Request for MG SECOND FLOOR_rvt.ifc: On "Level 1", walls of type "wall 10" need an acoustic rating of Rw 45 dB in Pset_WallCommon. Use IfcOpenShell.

First a look at what the model holds.

```python
import ifcopenshell
import ifcopenshell.util.element

model = ifcopenshell.open("MG SECOND FLOOR_rvt.ifc")
print(model.schema)
storey = next(s for s in model.by_type("IfcBuildingStorey") if s.Name == "Level 1")
walls = [e for e in ifcopenshell.util.element.get_decomposition(storey) if e.is_a("IfcWall")]
seen = {}
for e in walls:
    element_type = ifcopenshell.util.element.get_type(e)
    key = (element_type.Name if element_type != e and element_type else None, ifcopenshell.util.element.get_pset(e, "Pset_WallCommon", "AcousticRating"))
    seen[key] = seen.get(key, 0) + 1
for (name, value), count in sorted(seen.items(), key=str):
    print(count, "x", name, "|", value)
```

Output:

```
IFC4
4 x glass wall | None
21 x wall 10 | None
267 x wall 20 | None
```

```python
import ifcopenshell
import ifcopenshell.api.pset
import ifcopenshell.util.element

model = ifcopenshell.open("MG SECOND FLOOR_rvt.ifc")

storey = next(s for s in model.by_type("IfcBuildingStorey") if s.Name == "Level 1")
walls = [e for e in ifcopenshell.util.element.get_decomposition(storey) if e.is_a("IfcWall")]

count = 0
for e in walls:
    element_type = ifcopenshell.util.element.get_type(e)
    if element_type in (None, e) or element_type.Name != "wall 10":
        continue
    # add_pset returns the element's existing set when there is one.
    pset = ifcopenshell.api.pset.add_pset(model, product=e, name="Pset_WallCommon")
    ifcopenshell.api.pset.edit_pset(model, pset=pset, properties={"AcousticRating": "Rw 45 dB"})
    count += 1

print(count, "walls updated")

model.write("MG SECOND FLOOR_rvt_rev.ifc")
```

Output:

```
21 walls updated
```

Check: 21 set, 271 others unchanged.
